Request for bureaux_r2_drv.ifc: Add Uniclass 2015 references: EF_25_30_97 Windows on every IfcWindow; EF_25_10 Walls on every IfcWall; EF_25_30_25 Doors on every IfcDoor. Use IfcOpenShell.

First a look at what the model holds.

```python
import ifcopenshell

model = ifcopenshell.open("bureaux_r2_drv.ifc")
print(model.schema)
print("classifications:", [c.Name for c in model.by_type("IfcClassification")])
for ifc_class in ("IfcDoor", "IfcRoof", "IfcStair", "IfcWall", "IfcWindow"):
    print(ifc_class, len(model.by_type(ifc_class)))
```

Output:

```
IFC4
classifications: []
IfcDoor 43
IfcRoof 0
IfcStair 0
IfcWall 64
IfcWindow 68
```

```python
import ifcopenshell
import ifcopenshell.api.classification

model = ifcopenshell.open("bureaux_r2_drv.ifc")

system = ifcopenshell.api.classification.add_classification(model, classification="Uniclass 2015")

codes = {
    "IfcWindow": ("EF_25_30_97", "Windows"),
    "IfcWall": ("EF_25_10", "Walls"),
    "IfcDoor": ("EF_25_30_25", "Doors"),
}
for ifc_class, (code, name) in codes.items():
    products = model.by_type(ifc_class)
    ifcopenshell.api.classification.add_reference(
        model, products=products, classification=system, identification=code, name=name
    )
    print(code, len(products))

model.write("bureaux_r2_drv_v2.ifc")
```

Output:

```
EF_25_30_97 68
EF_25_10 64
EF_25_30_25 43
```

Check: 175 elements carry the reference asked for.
